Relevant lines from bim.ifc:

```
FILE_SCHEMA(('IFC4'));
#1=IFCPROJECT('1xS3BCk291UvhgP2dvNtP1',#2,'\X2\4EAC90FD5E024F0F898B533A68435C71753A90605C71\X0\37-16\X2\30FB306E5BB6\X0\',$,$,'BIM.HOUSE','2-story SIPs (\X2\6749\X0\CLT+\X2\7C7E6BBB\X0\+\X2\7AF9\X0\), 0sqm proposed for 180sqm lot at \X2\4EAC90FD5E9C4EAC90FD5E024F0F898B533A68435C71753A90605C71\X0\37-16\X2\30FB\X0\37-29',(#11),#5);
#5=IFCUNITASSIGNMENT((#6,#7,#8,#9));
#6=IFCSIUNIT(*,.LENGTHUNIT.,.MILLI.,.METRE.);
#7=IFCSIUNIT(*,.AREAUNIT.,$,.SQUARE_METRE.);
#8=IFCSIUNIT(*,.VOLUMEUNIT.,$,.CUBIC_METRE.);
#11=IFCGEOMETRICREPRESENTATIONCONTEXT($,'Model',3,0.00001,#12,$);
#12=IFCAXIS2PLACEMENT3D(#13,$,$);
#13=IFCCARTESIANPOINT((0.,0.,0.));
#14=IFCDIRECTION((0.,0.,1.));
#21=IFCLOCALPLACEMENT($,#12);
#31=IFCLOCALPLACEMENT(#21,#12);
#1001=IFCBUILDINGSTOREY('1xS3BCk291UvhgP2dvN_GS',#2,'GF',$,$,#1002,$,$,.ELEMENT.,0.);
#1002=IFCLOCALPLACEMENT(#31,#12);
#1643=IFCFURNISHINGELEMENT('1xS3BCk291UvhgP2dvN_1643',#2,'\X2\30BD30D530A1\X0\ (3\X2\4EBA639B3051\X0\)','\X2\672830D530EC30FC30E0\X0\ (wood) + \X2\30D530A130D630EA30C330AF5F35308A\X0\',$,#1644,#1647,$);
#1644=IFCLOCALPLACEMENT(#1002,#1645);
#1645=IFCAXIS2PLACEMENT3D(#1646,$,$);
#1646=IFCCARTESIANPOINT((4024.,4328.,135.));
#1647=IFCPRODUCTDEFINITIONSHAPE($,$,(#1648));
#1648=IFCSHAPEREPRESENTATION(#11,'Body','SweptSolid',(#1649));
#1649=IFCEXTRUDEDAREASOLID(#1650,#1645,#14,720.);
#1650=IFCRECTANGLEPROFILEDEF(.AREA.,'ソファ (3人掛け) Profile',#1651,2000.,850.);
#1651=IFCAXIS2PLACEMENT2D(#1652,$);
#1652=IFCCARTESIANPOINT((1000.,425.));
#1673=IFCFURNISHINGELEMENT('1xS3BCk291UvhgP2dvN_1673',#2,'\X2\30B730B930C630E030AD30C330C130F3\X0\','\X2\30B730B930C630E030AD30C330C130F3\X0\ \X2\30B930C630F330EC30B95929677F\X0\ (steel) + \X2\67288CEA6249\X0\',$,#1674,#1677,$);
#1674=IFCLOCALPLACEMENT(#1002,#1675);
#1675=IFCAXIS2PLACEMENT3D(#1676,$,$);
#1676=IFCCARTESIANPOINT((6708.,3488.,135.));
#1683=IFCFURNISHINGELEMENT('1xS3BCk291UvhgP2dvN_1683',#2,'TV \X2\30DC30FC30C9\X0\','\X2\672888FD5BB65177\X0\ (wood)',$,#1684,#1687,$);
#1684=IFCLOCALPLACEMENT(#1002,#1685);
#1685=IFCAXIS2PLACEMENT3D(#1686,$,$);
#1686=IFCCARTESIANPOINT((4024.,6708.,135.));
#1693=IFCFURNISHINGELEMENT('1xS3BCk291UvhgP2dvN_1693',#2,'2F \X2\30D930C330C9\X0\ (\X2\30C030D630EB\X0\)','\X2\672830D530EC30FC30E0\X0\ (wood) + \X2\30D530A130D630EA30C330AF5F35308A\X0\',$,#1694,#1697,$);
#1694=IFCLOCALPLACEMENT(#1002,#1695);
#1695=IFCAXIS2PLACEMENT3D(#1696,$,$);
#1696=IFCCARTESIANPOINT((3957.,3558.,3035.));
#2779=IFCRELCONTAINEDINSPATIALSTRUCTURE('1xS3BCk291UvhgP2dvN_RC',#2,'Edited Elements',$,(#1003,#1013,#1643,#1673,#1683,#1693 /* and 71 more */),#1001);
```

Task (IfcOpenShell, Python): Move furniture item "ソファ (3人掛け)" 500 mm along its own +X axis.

```python
import ifcopenshell
import ifcopenshell.api.geometry
import ifcopenshell.util.placement
import ifcopenshell.util.unit

model = ifcopenshell.open("bim.ifc")
unit_scale = ifcopenshell.util.unit.calculate_unit_scale(model)

item = model.by_guid("1xS3BCk291UvhgP2dvN_1643")
matrix = ifcopenshell.util.placement.get_local_placement(item.ObjectPlacement)
matrix[:3, 3] += matrix[:3, 0] * 0.5 / unit_scale
ifcopenshell.api.geometry.edit_object_placement(model, product=item, matrix=matrix, is_si=False)

print(ifcopenshell.util.placement.get_local_placement(item.ObjectPlacement).round(3) + 0.0)

model.write("bim_edited.ifc")
```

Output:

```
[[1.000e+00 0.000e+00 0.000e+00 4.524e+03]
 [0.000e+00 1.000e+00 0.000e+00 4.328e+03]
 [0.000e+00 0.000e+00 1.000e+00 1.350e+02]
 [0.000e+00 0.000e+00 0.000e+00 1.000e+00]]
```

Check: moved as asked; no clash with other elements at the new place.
